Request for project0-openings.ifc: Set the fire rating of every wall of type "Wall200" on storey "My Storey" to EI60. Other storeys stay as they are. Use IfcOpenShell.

First a look at what the model holds.

```python
import ifcopenshell
import ifcopenshell.util.element

model = ifcopenshell.open("project0-openings.ifc")
print(model.schema)
storey = next(s for s in model.by_type("IfcBuildingStorey") if s.Name == "My Storey")
walls = [e for e in ifcopenshell.util.element.get_decomposition(storey) if e.is_a("IfcWall")]
seen = {}
for e in walls:
    element_type = ifcopenshell.util.element.get_type(e)
    key = (element_type.Name if element_type != e and element_type else None, ifcopenshell.util.element.get_pset(e, "Pset_WallCommon", "FireRating"))
    seen[key] = seen.get(key, 0) + 1
for (name, value), count in sorted(seen.items(), key=str):
    print(count, "x", name, "|", value)
```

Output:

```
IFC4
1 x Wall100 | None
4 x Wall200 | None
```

```python
import ifcopenshell
import ifcopenshell.api.pset
import ifcopenshell.util.element

model = ifcopenshell.open("project0-openings.ifc")

storey = next(s for s in model.by_type("IfcBuildingStorey") if s.Name == "My Storey")
walls = [e for e in ifcopenshell.util.element.get_decomposition(storey) if e.is_a("IfcWall")]

count = 0
for e in walls:
    element_type = ifcopenshell.util.element.get_type(e)
    if element_type in (None, e) or element_type.Name != "Wall200":
        continue
    # add_pset returns the element's existing set when there is one.
    pset = ifcopenshell.api.pset.add_pset(model, product=e, name="Pset_WallCommon")
    ifcopenshell.api.pset.edit_pset(model, pset=pset, properties={"FireRating": "EI60"})
    count += 1

print(count, "walls updated")

model.write("project0-openings_rev.ifc")
```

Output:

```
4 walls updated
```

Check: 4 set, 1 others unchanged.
